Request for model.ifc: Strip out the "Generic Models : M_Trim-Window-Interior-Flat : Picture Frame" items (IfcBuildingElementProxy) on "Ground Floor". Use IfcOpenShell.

First a look at what the model holds.

```python
import ifcopenshell
import ifcopenshell.util.element

model = ifcopenshell.open("model.ifc")
print(model.schema)
storey = next(s for s in model.by_type("IfcBuildingStorey") if s.Name == "Ground Floor")
proxies = [e for e in ifcopenshell.util.element.get_decomposition(storey) if e.is_a("IfcBuildingElementProxy")]
seen = {}
for e in proxies:
    element_type = ifcopenshell.util.element.get_type(e)
    name = element_type.Name if element_type not in (None, e) else None
    seen[name] = seen.get(name, 0) + 1
for name, count in sorted(seen.items(), key=str):
    print(count, "x", name)
```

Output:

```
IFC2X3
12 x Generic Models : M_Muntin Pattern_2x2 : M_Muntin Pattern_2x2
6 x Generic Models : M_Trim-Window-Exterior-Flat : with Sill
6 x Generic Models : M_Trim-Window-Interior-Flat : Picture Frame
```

```python
import ifcopenshell
import ifcopenshell.api.root
import ifcopenshell.util.element

model = ifcopenshell.open("model.ifc")

storey = next(s for s in model.by_type("IfcBuildingStorey") if s.Name == "Ground Floor")
proxies = [e for e in ifcopenshell.util.element.get_decomposition(storey) if e.is_a("IfcBuildingElementProxy")]
targets = [e for e in proxies if (t := ifcopenshell.util.element.get_type(e)) not in (None, e) and t.Name == "Generic Models : M_Trim-Window-Interior-Flat : Picture Frame"]

for e in targets:
    ifcopenshell.api.root.remove_product(model, product=e)
print(len(targets), "removed")

model.write("model_edited.ifc")
```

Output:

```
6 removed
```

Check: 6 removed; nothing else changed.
